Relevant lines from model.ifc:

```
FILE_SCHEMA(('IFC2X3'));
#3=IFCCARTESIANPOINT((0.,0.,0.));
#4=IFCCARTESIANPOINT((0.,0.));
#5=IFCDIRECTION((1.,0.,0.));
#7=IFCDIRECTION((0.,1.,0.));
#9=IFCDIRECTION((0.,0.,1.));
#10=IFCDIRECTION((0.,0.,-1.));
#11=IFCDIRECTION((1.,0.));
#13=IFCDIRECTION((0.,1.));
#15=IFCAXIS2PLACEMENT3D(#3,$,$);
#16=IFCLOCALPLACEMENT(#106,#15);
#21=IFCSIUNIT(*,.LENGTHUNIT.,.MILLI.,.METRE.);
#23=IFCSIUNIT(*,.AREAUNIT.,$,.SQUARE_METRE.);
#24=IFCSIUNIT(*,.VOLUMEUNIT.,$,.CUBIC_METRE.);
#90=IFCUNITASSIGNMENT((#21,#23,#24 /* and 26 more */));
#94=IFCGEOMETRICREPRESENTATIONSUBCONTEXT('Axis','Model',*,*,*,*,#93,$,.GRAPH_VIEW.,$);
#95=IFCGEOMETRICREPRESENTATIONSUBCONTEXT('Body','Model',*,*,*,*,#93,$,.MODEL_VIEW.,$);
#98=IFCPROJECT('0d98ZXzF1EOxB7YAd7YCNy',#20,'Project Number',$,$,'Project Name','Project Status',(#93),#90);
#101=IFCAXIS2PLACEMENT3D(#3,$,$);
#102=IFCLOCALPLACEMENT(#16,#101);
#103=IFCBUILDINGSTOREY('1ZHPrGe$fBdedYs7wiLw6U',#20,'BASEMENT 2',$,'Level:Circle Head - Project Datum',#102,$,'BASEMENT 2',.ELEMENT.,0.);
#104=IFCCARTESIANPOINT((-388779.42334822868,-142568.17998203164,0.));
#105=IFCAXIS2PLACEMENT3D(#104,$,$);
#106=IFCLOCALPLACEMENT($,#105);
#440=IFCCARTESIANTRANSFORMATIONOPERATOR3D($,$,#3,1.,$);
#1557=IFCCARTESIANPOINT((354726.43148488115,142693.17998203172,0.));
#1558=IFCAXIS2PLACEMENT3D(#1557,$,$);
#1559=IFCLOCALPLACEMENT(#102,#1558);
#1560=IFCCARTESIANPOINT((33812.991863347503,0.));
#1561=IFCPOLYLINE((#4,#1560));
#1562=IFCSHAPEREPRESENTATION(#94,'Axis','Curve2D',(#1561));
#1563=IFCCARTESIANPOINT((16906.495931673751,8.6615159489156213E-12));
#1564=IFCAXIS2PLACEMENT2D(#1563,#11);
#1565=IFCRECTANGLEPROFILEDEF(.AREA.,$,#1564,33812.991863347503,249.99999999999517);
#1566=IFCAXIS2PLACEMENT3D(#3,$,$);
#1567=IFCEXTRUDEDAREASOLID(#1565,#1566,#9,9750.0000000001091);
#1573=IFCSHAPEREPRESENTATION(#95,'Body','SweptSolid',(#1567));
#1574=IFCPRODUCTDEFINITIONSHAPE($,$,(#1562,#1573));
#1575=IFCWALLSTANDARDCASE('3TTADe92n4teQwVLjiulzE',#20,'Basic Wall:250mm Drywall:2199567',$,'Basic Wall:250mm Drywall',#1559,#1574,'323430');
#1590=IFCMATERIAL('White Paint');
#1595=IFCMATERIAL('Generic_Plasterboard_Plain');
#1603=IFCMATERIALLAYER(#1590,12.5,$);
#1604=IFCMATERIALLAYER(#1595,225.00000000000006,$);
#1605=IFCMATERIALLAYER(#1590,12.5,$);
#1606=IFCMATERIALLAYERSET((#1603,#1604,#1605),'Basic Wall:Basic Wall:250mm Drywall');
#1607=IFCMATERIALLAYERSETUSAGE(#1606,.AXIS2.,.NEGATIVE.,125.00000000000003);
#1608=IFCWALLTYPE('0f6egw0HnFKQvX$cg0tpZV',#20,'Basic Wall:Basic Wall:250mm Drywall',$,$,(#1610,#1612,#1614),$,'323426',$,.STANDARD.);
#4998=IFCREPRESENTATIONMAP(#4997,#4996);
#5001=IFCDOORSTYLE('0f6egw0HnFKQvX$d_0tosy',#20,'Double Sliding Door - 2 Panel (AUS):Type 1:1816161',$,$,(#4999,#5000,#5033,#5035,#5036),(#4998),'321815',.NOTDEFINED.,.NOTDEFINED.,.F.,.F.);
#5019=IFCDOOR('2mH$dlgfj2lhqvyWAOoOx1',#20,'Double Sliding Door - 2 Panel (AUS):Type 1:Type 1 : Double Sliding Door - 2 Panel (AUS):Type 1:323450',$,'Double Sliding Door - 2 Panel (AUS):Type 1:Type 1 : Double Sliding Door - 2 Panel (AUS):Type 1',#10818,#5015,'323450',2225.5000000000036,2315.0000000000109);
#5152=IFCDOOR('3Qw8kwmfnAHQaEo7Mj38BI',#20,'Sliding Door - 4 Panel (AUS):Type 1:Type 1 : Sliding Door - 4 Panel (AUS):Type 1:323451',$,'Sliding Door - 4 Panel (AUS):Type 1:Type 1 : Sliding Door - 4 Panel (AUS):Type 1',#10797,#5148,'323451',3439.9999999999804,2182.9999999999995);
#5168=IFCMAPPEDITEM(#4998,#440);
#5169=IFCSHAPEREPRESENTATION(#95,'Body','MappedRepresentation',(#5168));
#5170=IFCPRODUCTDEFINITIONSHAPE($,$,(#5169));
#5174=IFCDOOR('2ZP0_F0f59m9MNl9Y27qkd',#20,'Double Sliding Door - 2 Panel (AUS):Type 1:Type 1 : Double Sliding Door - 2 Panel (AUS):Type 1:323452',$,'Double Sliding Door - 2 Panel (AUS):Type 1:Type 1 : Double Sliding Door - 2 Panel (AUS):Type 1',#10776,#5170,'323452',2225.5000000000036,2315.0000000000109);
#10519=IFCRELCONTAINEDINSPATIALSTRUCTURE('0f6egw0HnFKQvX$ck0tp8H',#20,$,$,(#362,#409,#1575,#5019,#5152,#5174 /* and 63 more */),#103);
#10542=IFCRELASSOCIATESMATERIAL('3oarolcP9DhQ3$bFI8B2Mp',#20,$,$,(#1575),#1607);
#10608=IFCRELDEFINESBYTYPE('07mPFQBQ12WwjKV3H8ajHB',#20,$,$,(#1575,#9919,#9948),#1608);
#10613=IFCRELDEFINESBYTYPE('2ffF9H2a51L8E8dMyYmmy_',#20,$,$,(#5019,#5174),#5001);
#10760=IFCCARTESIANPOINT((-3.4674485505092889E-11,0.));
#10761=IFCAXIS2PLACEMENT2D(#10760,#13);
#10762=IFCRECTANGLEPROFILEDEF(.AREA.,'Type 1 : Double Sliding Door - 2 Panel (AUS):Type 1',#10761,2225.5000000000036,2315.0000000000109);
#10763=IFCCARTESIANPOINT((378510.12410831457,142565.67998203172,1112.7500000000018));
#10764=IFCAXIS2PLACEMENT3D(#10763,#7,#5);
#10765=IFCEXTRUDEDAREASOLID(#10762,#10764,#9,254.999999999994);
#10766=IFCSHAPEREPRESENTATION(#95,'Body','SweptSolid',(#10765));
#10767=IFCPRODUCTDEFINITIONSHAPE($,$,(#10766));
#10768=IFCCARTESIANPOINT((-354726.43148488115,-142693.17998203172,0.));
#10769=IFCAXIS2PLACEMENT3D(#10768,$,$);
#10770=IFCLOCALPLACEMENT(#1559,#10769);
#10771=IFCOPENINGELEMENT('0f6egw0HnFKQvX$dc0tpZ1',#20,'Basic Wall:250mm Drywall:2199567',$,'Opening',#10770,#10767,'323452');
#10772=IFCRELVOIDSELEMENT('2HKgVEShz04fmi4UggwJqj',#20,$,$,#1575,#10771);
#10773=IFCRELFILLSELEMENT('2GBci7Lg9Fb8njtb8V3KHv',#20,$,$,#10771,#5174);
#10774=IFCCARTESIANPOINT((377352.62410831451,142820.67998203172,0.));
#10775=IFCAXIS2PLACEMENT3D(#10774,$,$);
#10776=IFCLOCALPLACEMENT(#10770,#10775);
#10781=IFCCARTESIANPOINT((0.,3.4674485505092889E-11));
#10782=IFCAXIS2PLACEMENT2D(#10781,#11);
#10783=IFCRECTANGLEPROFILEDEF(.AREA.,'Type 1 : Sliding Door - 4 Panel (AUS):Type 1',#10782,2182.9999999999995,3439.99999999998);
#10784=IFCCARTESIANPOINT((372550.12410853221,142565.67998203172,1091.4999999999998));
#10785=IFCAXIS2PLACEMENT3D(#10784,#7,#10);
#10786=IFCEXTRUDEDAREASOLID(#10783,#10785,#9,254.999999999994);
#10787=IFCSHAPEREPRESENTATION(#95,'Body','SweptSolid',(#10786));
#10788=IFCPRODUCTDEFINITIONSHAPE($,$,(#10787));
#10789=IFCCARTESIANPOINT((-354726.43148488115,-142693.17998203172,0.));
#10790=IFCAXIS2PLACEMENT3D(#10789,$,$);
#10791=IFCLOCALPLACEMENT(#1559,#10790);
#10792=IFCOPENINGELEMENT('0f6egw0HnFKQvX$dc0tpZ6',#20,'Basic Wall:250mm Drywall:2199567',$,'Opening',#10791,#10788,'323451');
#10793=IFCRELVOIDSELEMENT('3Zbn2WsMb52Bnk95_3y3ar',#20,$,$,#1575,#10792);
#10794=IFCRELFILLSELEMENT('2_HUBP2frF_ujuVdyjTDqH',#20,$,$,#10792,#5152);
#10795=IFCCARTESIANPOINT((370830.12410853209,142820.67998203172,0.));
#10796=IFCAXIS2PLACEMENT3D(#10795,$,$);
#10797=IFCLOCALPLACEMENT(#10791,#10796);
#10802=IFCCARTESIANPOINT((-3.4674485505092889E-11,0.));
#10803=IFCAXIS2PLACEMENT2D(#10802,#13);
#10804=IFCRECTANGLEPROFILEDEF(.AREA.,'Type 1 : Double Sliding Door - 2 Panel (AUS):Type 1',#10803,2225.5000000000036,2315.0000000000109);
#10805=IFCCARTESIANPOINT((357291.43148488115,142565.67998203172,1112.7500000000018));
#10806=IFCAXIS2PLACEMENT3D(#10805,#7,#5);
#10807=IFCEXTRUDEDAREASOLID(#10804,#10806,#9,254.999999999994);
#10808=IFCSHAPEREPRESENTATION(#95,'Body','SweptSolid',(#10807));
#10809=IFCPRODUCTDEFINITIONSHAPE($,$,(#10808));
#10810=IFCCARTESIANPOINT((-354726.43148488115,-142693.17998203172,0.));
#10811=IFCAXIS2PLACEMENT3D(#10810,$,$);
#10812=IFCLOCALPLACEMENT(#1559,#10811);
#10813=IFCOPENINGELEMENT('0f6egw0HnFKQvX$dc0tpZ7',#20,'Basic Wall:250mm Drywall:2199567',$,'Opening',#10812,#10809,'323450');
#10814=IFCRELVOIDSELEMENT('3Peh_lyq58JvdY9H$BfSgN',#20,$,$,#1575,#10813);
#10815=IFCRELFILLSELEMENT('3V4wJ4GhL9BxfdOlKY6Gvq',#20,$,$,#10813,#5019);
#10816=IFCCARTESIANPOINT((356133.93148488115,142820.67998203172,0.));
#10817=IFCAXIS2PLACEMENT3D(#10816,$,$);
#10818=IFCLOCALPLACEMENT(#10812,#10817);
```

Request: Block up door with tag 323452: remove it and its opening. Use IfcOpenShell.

```python
import ifcopenshell
import ifcopenshell.api.feature
import ifcopenshell.api.root
import ifcopenshell.geom
import ifcopenshell.util.shape

model = ifcopenshell.open("model.ifc")
settings = ifcopenshell.geom.settings()


def volume(element):
    """Net volume in cubic metres, openings subtracted."""
    shape = ifcopenshell.geom.create_shape(settings, element)
    return ifcopenshell.util.shape.get_volume(shape.geometry)


door = model.by_guid("2ZP0_F0f59m9MNl9Y27qkd")
opening = door.FillsVoids[0].RelatingOpeningElement
wall = opening.VoidsElements[0].RelatingBuildingElement
before = volume(wall)

ifcopenshell.api.root.remove_product(model, product=door)
ifcopenshell.api.feature.remove_feature(model, feature=opening)

after = volume(wall)

print(f"wall volume {before:.3f} -> {after:.3f} m3")

model.write("model_updated.ifc")
```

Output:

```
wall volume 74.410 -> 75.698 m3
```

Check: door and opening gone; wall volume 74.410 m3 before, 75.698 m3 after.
